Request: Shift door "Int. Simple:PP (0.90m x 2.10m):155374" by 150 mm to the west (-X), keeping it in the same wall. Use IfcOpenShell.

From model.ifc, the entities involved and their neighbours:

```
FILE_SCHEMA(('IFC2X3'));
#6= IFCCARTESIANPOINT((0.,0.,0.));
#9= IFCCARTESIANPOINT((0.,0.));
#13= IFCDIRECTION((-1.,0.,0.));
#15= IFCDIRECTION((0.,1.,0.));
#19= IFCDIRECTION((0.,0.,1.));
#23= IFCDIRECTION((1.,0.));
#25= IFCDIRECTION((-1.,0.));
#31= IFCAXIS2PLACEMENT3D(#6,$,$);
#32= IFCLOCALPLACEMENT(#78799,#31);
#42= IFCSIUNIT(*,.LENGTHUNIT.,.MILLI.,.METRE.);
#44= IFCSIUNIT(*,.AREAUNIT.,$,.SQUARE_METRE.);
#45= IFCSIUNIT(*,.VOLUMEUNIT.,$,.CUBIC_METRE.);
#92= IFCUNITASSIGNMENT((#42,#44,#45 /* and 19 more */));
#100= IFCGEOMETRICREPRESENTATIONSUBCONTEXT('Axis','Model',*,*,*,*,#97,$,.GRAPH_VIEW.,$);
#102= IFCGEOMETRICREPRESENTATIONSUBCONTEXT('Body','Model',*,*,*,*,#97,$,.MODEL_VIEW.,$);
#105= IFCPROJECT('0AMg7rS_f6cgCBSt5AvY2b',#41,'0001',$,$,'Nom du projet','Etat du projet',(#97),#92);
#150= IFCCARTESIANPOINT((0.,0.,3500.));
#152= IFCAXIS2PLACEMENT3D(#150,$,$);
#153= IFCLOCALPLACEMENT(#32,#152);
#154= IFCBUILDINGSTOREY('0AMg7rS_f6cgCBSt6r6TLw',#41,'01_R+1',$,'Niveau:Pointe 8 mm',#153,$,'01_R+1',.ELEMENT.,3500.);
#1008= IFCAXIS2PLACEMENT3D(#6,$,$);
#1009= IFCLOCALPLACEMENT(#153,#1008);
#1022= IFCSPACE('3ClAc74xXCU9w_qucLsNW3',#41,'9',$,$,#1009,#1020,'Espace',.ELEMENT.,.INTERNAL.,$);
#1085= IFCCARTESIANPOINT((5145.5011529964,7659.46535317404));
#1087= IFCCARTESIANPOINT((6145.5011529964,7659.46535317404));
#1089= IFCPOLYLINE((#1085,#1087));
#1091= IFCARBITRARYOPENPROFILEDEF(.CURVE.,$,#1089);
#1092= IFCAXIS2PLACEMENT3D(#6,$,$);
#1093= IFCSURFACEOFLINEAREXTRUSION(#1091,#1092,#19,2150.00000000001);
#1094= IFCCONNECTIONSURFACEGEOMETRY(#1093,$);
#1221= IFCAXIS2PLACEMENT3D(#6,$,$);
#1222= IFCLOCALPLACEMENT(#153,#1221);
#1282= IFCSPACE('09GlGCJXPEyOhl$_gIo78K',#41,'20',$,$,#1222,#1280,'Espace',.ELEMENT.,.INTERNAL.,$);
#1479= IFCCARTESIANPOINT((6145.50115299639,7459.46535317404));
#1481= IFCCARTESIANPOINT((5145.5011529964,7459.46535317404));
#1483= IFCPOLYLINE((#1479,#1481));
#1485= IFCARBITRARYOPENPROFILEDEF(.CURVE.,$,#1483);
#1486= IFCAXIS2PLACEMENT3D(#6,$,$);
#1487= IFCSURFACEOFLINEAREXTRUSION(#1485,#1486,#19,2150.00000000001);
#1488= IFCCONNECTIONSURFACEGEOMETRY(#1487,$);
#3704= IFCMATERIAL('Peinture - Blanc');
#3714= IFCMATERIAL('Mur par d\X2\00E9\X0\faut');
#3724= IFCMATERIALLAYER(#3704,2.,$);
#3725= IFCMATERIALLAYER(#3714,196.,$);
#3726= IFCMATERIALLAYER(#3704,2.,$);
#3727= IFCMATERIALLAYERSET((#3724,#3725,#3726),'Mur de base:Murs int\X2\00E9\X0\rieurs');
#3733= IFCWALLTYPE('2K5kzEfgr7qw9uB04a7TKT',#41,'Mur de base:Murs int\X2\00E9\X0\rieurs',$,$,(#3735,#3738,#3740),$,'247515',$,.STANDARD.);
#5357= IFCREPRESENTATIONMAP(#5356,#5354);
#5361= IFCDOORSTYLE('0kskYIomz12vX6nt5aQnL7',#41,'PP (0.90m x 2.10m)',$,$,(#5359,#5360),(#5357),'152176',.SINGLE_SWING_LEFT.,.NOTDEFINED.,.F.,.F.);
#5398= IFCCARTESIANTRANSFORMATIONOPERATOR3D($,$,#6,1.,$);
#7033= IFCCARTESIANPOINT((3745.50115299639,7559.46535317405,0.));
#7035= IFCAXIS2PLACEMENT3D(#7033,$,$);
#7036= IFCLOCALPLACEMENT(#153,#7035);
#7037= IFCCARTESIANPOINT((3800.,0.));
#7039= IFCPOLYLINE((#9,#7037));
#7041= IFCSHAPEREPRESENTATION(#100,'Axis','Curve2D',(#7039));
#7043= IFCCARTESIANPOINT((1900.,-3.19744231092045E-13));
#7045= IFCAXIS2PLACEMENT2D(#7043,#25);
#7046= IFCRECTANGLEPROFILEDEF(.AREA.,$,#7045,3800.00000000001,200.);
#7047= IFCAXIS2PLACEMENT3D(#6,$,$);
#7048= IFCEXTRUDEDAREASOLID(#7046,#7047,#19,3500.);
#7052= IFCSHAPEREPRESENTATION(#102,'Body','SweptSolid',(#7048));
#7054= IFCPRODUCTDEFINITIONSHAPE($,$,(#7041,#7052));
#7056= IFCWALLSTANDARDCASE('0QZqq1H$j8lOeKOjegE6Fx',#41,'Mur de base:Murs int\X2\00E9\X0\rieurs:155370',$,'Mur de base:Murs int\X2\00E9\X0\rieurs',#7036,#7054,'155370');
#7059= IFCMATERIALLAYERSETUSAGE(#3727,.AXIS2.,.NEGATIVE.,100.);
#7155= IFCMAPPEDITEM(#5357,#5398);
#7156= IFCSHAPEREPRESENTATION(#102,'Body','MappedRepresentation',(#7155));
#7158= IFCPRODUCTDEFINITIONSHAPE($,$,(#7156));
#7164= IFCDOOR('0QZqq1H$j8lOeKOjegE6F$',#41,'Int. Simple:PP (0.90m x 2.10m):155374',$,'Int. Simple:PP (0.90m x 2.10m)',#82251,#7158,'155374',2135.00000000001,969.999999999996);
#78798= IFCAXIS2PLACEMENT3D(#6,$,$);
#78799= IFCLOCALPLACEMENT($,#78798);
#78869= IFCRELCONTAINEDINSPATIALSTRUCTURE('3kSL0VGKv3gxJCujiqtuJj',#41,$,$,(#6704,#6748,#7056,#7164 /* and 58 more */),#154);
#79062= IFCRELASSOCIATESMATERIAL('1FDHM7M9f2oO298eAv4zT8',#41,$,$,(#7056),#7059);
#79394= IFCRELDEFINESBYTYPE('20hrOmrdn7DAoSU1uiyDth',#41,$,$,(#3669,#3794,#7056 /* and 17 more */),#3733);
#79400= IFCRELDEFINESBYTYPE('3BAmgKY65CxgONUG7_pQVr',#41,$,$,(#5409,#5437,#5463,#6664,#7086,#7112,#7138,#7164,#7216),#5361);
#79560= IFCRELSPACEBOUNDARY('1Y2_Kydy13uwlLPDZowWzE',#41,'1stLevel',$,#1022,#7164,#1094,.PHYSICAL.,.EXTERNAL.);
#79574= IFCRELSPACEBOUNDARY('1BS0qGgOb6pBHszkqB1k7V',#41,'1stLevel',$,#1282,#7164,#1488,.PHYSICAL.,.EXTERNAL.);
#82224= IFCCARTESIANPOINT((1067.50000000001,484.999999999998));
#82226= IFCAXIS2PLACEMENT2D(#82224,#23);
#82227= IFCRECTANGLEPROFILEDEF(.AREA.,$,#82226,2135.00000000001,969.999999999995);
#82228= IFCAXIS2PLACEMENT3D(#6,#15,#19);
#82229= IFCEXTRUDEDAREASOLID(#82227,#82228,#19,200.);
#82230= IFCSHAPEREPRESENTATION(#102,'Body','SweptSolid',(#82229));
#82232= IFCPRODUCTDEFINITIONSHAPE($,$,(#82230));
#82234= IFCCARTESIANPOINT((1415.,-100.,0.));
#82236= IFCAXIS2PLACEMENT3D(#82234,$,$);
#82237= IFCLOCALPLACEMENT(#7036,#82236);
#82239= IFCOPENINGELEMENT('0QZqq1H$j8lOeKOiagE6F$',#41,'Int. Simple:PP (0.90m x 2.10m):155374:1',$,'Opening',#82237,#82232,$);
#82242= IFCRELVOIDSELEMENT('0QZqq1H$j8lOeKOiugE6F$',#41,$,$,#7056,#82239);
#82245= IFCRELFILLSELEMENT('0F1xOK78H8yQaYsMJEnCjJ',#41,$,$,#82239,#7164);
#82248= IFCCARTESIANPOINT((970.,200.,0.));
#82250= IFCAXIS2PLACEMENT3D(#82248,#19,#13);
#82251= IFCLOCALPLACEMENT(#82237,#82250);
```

```python
import numpy as np
import ifcopenshell
import ifcopenshell.api.geometry
import ifcopenshell.util.placement
import ifcopenshell.util.unit

model = ifcopenshell.open("model.ifc")
unit_scale = ifcopenshell.util.unit.calculate_unit_scale(model)

door = model.by_guid("0QZqq1H$j8lOeKOjegE6F$")
opening = door.FillsVoids[0].RelatingOpeningElement
wall = opening.VoidsElements[0].RelatingBuildingElement

wall_matrix = ifcopenshell.util.placement.get_local_placement(wall.ObjectPlacement)
shift = wall_matrix[:3, 0] * -0.15 / unit_scale
before = ifcopenshell.util.placement.get_local_placement(door.ObjectPlacement)[:3, 3].copy()

# The door is placed relative to its opening, so it follows when the opening moves.
matrix = ifcopenshell.util.placement.get_local_placement(opening.ObjectPlacement)
matrix[:3, 3] += shift
ifcopenshell.api.geometry.edit_object_placement(
    model, product=opening, matrix=matrix, is_si=False, should_transform_children=True
)

# Space boundary surfaces are stored in each space's coordinates; move them too.
for rel in door.ProvidesBoundaries:
    if not rel.ConnectionGeometry:
        continue
    surface = rel.ConnectionGeometry.SurfaceOnRelatingElement
    space_matrix = ifcopenshell.util.placement.get_local_placement(rel.RelatingSpace.ObjectPlacement)
    point = np.array(surface.Position.Location.Coordinates) + space_matrix[:3, :3].T @ shift
    surface.Position = model.createIfcAxis2Placement3D(
        model.createIfcCartesianPoint(point.tolist()), surface.Position.Axis, surface.Position.RefDirection
    )

after = ifcopenshell.util.placement.get_local_placement(door.ObjectPlacement)[:3, 3]
print("door moved by", (after - before).round(3) + 0.0)

model.write("model_v2.ifc")
```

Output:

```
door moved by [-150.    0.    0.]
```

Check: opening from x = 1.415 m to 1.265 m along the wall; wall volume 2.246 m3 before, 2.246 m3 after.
